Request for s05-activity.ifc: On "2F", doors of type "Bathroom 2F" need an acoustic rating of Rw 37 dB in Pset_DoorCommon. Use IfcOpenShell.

First a look at what the model holds.

```python
import ifcopenshell
import ifcopenshell.util.element

model = ifcopenshell.open("s05-activity.ifc")
print(model.schema)
storey = next(s for s in model.by_type("IfcBuildingStorey") if s.Name == "2F")
doors = [e for e in ifcopenshell.util.element.get_decomposition(storey) if e.is_a("IfcDoor")]
seen = {}
for e in doors:
    element_type = ifcopenshell.util.element.get_type(e)
    key = (element_type.Name if element_type != e and element_type else None, ifcopenshell.util.element.get_pset(e, "Pset_DoorCommon", "AcousticRating"))
    seen[key] = seen.get(key, 0) + 1
for (name, value), count in sorted(seen.items(), key=str):
    print(count, "x", name, "|", value)
```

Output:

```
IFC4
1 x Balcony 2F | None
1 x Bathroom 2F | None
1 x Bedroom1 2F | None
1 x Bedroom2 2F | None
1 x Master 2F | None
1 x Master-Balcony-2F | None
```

```python
import ifcopenshell
import ifcopenshell.api.pset
import ifcopenshell.util.element

model = ifcopenshell.open("s05-activity.ifc")

storey = next(s for s in model.by_type("IfcBuildingStorey") if s.Name == "2F")
doors = [e for e in ifcopenshell.util.element.get_decomposition(storey) if e.is_a("IfcDoor")]

count = 0
for e in doors:
    element_type = ifcopenshell.util.element.get_type(e)
    if element_type in (None, e) or element_type.Name != "Bathroom 2F":
        continue
    # add_pset returns the element's existing set when there is one.
    pset = ifcopenshell.api.pset.add_pset(model, product=e, name="Pset_DoorCommon")
    ifcopenshell.api.pset.edit_pset(model, pset=pset, properties={"AcousticRating": "Rw 37 dB"})
    count += 1

print(count, "doors updated")

model.write("s05-activity_rev.ifc")
```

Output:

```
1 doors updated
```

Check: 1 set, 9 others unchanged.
